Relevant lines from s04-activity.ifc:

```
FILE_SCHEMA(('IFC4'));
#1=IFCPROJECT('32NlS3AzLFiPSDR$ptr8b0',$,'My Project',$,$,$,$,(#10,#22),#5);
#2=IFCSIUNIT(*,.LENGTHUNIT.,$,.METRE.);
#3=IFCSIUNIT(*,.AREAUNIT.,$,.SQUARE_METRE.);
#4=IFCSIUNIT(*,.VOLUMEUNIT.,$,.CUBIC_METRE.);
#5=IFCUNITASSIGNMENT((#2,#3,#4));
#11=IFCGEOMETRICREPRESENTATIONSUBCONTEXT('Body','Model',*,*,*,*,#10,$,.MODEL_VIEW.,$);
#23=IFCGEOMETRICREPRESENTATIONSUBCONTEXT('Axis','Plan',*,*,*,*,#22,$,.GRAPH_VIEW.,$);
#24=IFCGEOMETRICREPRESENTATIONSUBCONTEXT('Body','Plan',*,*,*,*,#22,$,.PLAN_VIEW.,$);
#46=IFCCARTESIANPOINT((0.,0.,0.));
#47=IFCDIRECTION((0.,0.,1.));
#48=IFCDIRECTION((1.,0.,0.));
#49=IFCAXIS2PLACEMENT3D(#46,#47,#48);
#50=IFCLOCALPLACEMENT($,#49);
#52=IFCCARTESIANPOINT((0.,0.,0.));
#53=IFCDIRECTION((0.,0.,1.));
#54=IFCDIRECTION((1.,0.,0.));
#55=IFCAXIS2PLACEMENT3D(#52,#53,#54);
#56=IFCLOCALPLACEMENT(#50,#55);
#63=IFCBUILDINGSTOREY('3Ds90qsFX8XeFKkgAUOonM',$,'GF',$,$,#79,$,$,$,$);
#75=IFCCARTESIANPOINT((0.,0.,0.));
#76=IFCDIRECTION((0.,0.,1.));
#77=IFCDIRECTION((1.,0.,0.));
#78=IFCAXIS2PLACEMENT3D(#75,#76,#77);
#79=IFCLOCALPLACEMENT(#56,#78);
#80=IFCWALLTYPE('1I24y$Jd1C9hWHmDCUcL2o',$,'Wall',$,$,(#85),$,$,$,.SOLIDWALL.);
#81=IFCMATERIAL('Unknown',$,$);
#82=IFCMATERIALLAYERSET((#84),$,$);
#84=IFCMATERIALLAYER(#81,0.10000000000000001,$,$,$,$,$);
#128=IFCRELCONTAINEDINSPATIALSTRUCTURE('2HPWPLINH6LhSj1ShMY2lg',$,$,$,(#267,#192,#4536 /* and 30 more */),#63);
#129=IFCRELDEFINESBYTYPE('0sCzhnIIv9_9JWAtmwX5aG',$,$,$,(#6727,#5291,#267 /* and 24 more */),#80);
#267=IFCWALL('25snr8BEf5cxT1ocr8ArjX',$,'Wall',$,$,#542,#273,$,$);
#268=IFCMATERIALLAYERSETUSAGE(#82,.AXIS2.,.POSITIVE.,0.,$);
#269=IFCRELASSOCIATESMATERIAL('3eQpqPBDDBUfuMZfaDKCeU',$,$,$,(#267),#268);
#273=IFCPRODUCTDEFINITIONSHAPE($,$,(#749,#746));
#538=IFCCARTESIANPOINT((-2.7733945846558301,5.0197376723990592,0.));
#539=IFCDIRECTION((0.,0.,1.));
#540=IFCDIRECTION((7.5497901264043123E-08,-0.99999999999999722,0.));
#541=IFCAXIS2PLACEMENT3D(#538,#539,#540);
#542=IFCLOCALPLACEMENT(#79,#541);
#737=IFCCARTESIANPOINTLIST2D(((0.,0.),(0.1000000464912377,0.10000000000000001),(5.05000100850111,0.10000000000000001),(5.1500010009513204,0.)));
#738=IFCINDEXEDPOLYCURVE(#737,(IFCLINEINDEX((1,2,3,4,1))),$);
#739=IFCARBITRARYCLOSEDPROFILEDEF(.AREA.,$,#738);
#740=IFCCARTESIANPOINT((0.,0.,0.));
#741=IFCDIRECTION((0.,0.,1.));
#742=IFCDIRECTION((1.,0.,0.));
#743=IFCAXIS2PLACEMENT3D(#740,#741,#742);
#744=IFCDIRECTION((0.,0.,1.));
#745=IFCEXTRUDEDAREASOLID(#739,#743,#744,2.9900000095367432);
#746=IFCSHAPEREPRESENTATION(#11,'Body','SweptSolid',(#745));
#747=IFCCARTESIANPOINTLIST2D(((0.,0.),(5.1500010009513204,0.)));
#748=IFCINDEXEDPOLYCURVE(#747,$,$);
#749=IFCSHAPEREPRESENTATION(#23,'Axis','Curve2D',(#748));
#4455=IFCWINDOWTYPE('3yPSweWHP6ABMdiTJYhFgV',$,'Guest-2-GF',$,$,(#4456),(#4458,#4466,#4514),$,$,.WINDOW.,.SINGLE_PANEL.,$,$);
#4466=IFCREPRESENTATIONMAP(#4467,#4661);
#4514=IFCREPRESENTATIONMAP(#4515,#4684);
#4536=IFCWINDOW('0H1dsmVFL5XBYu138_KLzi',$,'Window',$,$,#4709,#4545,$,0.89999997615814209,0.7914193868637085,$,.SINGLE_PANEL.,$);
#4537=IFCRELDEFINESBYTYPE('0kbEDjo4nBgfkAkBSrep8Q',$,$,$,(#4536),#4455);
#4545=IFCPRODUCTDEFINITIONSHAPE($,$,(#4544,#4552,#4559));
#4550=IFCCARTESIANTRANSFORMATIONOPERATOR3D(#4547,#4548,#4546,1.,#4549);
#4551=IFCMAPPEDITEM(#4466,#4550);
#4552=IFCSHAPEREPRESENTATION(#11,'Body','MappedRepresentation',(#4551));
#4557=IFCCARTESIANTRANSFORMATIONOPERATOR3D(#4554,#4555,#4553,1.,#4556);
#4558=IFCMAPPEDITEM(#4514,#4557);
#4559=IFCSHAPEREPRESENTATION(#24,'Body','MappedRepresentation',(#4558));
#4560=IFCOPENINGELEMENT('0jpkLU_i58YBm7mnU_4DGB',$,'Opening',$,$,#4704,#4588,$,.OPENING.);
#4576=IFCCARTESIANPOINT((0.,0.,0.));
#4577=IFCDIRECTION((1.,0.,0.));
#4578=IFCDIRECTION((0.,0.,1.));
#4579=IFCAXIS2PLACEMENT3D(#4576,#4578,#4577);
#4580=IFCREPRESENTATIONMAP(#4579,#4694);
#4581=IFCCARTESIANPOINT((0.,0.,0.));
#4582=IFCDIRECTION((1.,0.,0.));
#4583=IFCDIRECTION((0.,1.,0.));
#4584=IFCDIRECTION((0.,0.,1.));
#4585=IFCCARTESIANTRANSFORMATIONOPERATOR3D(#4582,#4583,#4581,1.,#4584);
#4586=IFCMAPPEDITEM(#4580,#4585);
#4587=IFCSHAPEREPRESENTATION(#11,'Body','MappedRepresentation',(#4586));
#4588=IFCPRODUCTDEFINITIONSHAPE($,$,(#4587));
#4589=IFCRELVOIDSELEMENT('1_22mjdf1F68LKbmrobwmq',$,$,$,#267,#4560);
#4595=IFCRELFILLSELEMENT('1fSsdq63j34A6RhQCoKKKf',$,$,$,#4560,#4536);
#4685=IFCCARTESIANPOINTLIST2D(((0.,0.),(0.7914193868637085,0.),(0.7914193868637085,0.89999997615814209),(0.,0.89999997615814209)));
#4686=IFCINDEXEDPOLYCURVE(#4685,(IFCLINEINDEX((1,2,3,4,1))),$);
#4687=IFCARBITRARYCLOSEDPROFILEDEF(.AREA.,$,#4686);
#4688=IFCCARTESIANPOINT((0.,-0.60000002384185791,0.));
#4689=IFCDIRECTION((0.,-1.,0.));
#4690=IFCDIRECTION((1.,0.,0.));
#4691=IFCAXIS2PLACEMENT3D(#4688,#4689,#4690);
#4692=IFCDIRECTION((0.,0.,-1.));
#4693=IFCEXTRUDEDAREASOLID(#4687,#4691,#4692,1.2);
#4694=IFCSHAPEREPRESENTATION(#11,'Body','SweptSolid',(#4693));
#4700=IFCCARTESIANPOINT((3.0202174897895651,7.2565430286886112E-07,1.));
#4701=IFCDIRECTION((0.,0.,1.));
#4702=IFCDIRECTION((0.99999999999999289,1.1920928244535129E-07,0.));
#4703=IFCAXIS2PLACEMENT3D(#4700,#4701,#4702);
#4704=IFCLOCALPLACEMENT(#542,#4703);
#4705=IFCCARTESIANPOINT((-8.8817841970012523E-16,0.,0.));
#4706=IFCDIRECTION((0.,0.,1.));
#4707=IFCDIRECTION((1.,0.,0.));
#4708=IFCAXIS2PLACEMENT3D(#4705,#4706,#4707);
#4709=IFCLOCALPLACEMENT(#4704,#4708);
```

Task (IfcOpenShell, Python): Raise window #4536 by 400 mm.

```python
import numpy as np
import ifcopenshell
import ifcopenshell.api.geometry
import ifcopenshell.util.placement
import ifcopenshell.util.unit

model = ifcopenshell.open("s04-activity.ifc")
unit_scale = ifcopenshell.util.unit.calculate_unit_scale(model)

window = model.by_id(4536)
opening = window.FillsVoids[0].RelatingOpeningElement
dz = 0.4

shift = np.array([0.0, 0.0, dz])
# The window is placed relative to its opening, so it follows when the opening moves.
matrix = ifcopenshell.util.placement.get_local_placement(opening.ObjectPlacement)
matrix[:3, 3] += shift
ifcopenshell.api.geometry.edit_object_placement(
    model, product=opening, matrix=matrix, is_si=False, should_transform_children=True
)

print(f"moved by {dz * unit_scale:+.3f} m")

model.write("s04-activity-out.ifc")
```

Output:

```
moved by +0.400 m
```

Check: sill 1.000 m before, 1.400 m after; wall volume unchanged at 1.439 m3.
